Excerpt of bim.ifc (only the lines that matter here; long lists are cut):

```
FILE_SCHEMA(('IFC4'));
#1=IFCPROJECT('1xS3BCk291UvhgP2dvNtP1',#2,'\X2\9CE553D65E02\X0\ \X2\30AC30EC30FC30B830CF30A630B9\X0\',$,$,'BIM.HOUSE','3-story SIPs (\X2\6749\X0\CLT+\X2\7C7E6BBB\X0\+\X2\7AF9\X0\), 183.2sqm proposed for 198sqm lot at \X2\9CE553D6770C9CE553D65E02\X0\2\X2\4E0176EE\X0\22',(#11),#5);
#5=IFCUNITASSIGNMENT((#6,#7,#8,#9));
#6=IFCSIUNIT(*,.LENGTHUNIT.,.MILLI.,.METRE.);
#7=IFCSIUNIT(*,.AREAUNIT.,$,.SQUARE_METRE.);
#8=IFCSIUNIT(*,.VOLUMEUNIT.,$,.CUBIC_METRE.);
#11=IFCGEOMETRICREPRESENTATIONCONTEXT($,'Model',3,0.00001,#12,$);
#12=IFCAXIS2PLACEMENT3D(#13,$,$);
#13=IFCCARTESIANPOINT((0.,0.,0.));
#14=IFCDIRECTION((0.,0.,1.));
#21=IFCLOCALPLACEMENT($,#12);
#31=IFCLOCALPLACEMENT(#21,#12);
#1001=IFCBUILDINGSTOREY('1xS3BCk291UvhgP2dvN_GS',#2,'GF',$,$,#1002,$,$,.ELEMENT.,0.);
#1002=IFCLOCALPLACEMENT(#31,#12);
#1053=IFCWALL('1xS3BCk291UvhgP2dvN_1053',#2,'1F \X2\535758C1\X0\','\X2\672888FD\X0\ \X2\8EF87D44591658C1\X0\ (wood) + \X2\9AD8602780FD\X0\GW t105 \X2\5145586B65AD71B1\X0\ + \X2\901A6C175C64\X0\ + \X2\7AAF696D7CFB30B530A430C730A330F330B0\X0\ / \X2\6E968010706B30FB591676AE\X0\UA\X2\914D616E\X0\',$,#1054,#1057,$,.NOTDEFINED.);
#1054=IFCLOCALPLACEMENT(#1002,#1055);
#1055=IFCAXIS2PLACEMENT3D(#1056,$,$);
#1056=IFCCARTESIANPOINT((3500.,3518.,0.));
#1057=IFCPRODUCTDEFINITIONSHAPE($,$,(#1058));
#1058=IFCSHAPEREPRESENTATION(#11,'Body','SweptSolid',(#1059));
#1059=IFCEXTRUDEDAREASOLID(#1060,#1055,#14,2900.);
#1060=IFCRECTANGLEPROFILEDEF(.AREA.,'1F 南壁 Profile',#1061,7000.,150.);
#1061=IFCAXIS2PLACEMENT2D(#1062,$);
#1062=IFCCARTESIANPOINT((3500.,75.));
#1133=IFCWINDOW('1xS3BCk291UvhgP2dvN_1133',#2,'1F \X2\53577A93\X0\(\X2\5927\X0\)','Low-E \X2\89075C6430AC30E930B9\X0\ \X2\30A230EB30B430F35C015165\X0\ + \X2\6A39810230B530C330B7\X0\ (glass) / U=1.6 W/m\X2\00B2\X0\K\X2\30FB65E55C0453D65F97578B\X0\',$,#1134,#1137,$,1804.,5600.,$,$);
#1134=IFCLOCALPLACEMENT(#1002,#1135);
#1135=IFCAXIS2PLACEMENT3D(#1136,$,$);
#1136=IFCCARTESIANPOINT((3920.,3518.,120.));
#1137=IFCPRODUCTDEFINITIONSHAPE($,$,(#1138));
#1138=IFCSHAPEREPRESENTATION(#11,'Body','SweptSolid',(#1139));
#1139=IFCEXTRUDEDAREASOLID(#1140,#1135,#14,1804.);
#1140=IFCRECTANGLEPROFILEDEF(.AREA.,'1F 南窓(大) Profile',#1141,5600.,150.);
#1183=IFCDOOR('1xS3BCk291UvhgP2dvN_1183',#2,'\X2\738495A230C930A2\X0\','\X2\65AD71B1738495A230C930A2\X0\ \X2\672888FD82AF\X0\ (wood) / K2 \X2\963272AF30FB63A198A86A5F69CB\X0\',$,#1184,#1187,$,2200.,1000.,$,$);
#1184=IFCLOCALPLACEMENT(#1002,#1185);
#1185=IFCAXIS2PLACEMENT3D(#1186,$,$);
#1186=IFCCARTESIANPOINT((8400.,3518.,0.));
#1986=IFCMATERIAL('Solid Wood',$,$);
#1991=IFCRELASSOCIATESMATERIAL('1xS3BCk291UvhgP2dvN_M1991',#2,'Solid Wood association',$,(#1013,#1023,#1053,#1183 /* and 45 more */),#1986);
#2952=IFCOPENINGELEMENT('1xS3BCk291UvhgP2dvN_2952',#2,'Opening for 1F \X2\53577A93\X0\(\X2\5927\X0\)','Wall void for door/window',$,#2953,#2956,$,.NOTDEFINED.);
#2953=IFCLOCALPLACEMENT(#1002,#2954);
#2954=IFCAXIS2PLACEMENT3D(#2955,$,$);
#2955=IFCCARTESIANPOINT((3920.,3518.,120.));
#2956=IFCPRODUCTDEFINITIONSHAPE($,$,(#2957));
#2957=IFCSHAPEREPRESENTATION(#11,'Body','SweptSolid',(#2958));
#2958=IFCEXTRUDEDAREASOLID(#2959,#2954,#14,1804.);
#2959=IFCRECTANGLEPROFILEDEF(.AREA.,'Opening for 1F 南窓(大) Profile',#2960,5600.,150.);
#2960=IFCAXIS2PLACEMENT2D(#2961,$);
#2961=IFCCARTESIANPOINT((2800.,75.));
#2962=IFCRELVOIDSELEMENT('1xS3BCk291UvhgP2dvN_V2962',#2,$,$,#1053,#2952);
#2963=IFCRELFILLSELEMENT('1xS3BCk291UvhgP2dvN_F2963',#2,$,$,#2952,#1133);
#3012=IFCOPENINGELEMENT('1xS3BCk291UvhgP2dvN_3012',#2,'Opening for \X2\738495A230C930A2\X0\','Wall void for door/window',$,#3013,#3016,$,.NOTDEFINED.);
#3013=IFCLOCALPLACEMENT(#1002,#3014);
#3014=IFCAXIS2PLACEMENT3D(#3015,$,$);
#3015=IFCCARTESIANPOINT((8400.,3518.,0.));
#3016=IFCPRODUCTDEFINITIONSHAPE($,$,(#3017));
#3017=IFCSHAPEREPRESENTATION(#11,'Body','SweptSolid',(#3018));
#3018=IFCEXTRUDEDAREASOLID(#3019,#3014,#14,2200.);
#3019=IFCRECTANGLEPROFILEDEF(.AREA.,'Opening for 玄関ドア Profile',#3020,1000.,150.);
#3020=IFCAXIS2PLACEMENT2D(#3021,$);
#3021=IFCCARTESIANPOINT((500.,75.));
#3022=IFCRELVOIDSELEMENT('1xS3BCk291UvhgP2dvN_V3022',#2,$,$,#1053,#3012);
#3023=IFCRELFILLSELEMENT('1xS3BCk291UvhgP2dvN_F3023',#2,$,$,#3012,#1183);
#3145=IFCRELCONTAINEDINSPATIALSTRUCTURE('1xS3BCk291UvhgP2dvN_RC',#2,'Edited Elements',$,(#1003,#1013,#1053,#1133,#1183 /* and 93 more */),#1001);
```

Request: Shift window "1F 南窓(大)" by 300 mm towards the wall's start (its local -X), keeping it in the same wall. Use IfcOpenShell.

```python
import ifcopenshell
import ifcopenshell.api.geometry
import ifcopenshell.util.placement
import ifcopenshell.util.unit

model = ifcopenshell.open("bim.ifc")
unit_scale = ifcopenshell.util.unit.calculate_unit_scale(model)

window = model.by_guid("1xS3BCk291UvhgP2dvN_1133")
opening = window.FillsVoids[0].RelatingOpeningElement
wall = opening.VoidsElements[0].RelatingBuildingElement

wall_matrix = ifcopenshell.util.placement.get_local_placement(wall.ObjectPlacement)
shift = wall_matrix[:3, 0] * -0.3 / unit_scale
before = ifcopenshell.util.placement.get_local_placement(window.ObjectPlacement)[:3, 3].copy()

# The window is not placed relative to its opening, so move both.
for product in (opening, window):
    matrix = ifcopenshell.util.placement.get_local_placement(product.ObjectPlacement)
    matrix[:3, 3] += shift
    ifcopenshell.api.geometry.edit_object_placement(model, product=product, matrix=matrix, is_si=False)

after = ifcopenshell.util.placement.get_local_placement(window.ObjectPlacement)[:3, 3]
print("window moved by", (after - before).round(3) + 0.0)

model.write("bim_v2.ifc")
```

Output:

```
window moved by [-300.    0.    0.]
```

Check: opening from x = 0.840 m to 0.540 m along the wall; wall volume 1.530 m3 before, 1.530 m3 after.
